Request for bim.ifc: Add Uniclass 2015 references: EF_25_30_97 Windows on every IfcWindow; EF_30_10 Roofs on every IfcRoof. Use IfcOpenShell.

First a look at what the model holds.

```python
import ifcopenshell

model = ifcopenshell.open("bim.ifc")
print(model.schema)
print("classifications:", [c.Name for c in model.by_type("IfcClassification")])
for ifc_class in ("IfcDoor", "IfcRoof", "IfcStair", "IfcWall", "IfcWindow"):
    print(ifc_class, len(model.by_type(ifc_class)))
```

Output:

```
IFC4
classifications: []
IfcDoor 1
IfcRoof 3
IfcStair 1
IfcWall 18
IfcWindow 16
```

```python
import ifcopenshell
import ifcopenshell.api.classification

model = ifcopenshell.open("bim.ifc")

system = ifcopenshell.api.classification.add_classification(model, classification="Uniclass 2015")

codes = {
    "IfcWindow": ("EF_25_30_97", "Windows"),
    "IfcRoof": ("EF_30_10", "Roofs"),
}
for ifc_class, (code, name) in codes.items():
    products = model.by_type(ifc_class)
    ifcopenshell.api.classification.add_reference(
        model, products=products, classification=system, identification=code, name=name
    )
    print(code, len(products))

model.write("bim_updated.ifc")
```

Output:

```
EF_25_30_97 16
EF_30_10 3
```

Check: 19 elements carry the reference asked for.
